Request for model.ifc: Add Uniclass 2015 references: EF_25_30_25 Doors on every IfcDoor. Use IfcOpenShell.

First a look at what the model holds.

```python
import ifcopenshell

model = ifcopenshell.open("model.ifc")
print(model.schema)
print("classifications:", [c.Name for c in model.by_type("IfcClassification")])
for ifc_class in ("IfcDoor", "IfcRoof", "IfcStair", "IfcWall", "IfcWindow"):
    print(ifc_class, len(model.by_type(ifc_class)))
```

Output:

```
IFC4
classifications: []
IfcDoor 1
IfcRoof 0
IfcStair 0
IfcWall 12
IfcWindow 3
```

```python
import ifcopenshell
import ifcopenshell.api.classification

model = ifcopenshell.open("model.ifc")

system = ifcopenshell.api.classification.add_classification(model, classification="Uniclass 2015")

codes = {
    "IfcDoor": ("EF_25_30_25", "Doors"),
}
for ifc_class, (code, name) in codes.items():
    products = model.by_type(ifc_class)
    ifcopenshell.api.classification.add_reference(
        model, products=products, classification=system, identification=code, name=name
    )
    print(code, len(products))

model.write("model_updated.ifc")
```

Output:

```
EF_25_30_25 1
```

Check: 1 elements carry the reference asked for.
